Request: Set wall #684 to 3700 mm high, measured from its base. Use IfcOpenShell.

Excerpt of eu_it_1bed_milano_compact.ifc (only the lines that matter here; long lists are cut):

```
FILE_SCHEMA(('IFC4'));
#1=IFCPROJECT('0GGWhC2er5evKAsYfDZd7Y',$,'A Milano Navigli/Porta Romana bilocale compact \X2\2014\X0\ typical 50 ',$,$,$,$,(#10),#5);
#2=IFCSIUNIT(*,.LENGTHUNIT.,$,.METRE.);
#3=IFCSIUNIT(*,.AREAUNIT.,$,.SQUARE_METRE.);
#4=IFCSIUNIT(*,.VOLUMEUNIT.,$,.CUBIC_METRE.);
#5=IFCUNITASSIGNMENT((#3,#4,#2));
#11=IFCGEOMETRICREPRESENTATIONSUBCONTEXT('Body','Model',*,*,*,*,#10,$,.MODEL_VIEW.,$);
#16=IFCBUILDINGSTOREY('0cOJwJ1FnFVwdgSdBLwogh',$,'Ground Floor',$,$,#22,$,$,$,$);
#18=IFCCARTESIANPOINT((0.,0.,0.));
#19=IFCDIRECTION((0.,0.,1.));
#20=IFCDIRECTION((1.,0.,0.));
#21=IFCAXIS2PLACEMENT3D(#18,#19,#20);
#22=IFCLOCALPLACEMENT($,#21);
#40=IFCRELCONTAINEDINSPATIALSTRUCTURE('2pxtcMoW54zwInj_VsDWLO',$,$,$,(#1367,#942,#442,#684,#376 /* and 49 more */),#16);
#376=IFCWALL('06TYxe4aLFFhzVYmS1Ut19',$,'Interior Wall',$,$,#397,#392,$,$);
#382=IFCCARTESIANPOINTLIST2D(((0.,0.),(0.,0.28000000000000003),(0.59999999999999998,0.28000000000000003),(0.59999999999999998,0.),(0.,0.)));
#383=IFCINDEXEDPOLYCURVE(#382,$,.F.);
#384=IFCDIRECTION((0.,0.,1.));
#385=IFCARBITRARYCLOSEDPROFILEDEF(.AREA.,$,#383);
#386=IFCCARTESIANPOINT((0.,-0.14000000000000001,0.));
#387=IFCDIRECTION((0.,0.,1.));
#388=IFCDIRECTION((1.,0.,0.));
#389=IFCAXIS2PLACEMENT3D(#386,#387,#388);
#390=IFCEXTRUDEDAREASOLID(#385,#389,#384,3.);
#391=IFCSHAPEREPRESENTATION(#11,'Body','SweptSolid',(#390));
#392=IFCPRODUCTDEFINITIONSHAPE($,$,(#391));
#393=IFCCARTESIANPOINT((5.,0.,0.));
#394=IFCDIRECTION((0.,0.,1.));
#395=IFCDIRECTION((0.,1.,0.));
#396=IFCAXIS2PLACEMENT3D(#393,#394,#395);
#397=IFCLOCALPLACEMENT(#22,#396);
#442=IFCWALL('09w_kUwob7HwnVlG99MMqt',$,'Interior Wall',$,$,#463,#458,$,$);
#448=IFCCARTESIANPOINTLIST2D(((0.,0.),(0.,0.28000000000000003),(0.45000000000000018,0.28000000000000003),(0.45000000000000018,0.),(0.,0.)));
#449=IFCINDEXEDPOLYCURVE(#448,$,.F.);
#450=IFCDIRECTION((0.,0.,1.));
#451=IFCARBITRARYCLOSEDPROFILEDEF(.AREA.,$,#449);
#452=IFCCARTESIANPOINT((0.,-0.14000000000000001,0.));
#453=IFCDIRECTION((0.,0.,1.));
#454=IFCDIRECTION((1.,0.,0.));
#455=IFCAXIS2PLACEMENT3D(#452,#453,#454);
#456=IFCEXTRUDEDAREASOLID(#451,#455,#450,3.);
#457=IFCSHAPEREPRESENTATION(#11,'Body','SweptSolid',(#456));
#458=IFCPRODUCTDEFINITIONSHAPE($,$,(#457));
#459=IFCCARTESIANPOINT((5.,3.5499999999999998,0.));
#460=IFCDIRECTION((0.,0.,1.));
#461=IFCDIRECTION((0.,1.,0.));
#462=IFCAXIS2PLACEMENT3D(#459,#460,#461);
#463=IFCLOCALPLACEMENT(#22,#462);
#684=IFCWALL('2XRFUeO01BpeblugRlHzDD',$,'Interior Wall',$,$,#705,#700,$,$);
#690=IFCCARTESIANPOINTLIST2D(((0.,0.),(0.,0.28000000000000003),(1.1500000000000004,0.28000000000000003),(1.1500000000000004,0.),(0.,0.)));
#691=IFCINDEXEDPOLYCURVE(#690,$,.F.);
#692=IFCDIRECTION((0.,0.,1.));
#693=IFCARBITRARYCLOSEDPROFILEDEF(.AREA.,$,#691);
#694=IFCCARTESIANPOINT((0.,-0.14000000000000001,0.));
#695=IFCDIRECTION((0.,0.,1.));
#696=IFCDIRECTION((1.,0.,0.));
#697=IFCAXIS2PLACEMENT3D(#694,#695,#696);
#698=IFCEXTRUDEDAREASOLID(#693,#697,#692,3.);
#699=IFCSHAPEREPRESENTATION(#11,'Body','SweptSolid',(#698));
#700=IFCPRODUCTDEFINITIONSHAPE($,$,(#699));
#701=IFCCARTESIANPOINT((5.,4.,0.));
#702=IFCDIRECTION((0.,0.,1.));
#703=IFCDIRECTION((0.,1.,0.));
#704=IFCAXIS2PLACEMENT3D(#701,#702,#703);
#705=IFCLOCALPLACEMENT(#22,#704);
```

```python
import ifcopenshell
import ifcopenshell.geom
import ifcopenshell.util.representation
import ifcopenshell.util.shape
import ifcopenshell.util.unit

model = ifcopenshell.open("eu_it_1bed_milano_compact.ifc")
unit_scale = ifcopenshell.util.unit.calculate_unit_scale(model)
settings = ifcopenshell.geom.settings()


def volume(element):
    """Net volume in cubic metres, openings subtracted."""
    shape = ifcopenshell.geom.create_shape(settings, element)
    return ifcopenshell.util.shape.get_volume(shape.geometry)


wall = model.by_guid("2XRFUeO01BpeblugRlHzDD")
before = volume(wall)

body = ifcopenshell.util.representation.get_representation(wall, "Model", "Body")
solid = body.Items[0]
old_height = solid.Depth
solid.Depth = 3.7 / unit_scale
after = volume(wall)

print(f"height {old_height:g} -> {solid.Depth:g}, volume {before:.3f} -> {after:.3f} m3")

model.write("eu_it_1bed_milano_compact-out.ifc")
```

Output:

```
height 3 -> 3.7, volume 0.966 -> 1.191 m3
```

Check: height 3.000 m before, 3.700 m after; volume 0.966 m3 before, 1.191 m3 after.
